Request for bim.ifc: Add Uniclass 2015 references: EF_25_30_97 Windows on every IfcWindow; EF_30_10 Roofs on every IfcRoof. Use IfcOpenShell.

First a look at what the model holds.

```python
import ifcopenshell

model = ifcopenshell.open("bim.ifc")
print(model.schema)
print("classifications:", [c.Name for c in model.by_type("IfcClassification")])
for ifc_class in ("IfcDoor", "IfcRoof", "IfcStair", "IfcWall", "IfcWindow"):
    print(ifc_class, len(model.by_type(ifc_class)))
```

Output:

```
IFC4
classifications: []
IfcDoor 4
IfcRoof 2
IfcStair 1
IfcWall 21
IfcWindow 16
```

```python
import ifcopenshell
import ifcopenshell.api.classification

model = ifcopenshell.open("bim.ifc")

system = ifcopenshell.api.classification.add_classification(model, classification="Uniclass 2015")

codes = {
    "IfcWindow": ("EF_25_30_97", "Windows"),
    "IfcRoof": ("EF_30_10", "Roofs"),
}
for ifc_class, (code, name) in codes.items():
    products = model.by_type(ifc_class)
    ifcopenshell.api.classification.add_reference(
        model, products=products, classification=system, identification=code, name=name
    )
    print(code, len(products))

model.write("bim_rev.ifc")
```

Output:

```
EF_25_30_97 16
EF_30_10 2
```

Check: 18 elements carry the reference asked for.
